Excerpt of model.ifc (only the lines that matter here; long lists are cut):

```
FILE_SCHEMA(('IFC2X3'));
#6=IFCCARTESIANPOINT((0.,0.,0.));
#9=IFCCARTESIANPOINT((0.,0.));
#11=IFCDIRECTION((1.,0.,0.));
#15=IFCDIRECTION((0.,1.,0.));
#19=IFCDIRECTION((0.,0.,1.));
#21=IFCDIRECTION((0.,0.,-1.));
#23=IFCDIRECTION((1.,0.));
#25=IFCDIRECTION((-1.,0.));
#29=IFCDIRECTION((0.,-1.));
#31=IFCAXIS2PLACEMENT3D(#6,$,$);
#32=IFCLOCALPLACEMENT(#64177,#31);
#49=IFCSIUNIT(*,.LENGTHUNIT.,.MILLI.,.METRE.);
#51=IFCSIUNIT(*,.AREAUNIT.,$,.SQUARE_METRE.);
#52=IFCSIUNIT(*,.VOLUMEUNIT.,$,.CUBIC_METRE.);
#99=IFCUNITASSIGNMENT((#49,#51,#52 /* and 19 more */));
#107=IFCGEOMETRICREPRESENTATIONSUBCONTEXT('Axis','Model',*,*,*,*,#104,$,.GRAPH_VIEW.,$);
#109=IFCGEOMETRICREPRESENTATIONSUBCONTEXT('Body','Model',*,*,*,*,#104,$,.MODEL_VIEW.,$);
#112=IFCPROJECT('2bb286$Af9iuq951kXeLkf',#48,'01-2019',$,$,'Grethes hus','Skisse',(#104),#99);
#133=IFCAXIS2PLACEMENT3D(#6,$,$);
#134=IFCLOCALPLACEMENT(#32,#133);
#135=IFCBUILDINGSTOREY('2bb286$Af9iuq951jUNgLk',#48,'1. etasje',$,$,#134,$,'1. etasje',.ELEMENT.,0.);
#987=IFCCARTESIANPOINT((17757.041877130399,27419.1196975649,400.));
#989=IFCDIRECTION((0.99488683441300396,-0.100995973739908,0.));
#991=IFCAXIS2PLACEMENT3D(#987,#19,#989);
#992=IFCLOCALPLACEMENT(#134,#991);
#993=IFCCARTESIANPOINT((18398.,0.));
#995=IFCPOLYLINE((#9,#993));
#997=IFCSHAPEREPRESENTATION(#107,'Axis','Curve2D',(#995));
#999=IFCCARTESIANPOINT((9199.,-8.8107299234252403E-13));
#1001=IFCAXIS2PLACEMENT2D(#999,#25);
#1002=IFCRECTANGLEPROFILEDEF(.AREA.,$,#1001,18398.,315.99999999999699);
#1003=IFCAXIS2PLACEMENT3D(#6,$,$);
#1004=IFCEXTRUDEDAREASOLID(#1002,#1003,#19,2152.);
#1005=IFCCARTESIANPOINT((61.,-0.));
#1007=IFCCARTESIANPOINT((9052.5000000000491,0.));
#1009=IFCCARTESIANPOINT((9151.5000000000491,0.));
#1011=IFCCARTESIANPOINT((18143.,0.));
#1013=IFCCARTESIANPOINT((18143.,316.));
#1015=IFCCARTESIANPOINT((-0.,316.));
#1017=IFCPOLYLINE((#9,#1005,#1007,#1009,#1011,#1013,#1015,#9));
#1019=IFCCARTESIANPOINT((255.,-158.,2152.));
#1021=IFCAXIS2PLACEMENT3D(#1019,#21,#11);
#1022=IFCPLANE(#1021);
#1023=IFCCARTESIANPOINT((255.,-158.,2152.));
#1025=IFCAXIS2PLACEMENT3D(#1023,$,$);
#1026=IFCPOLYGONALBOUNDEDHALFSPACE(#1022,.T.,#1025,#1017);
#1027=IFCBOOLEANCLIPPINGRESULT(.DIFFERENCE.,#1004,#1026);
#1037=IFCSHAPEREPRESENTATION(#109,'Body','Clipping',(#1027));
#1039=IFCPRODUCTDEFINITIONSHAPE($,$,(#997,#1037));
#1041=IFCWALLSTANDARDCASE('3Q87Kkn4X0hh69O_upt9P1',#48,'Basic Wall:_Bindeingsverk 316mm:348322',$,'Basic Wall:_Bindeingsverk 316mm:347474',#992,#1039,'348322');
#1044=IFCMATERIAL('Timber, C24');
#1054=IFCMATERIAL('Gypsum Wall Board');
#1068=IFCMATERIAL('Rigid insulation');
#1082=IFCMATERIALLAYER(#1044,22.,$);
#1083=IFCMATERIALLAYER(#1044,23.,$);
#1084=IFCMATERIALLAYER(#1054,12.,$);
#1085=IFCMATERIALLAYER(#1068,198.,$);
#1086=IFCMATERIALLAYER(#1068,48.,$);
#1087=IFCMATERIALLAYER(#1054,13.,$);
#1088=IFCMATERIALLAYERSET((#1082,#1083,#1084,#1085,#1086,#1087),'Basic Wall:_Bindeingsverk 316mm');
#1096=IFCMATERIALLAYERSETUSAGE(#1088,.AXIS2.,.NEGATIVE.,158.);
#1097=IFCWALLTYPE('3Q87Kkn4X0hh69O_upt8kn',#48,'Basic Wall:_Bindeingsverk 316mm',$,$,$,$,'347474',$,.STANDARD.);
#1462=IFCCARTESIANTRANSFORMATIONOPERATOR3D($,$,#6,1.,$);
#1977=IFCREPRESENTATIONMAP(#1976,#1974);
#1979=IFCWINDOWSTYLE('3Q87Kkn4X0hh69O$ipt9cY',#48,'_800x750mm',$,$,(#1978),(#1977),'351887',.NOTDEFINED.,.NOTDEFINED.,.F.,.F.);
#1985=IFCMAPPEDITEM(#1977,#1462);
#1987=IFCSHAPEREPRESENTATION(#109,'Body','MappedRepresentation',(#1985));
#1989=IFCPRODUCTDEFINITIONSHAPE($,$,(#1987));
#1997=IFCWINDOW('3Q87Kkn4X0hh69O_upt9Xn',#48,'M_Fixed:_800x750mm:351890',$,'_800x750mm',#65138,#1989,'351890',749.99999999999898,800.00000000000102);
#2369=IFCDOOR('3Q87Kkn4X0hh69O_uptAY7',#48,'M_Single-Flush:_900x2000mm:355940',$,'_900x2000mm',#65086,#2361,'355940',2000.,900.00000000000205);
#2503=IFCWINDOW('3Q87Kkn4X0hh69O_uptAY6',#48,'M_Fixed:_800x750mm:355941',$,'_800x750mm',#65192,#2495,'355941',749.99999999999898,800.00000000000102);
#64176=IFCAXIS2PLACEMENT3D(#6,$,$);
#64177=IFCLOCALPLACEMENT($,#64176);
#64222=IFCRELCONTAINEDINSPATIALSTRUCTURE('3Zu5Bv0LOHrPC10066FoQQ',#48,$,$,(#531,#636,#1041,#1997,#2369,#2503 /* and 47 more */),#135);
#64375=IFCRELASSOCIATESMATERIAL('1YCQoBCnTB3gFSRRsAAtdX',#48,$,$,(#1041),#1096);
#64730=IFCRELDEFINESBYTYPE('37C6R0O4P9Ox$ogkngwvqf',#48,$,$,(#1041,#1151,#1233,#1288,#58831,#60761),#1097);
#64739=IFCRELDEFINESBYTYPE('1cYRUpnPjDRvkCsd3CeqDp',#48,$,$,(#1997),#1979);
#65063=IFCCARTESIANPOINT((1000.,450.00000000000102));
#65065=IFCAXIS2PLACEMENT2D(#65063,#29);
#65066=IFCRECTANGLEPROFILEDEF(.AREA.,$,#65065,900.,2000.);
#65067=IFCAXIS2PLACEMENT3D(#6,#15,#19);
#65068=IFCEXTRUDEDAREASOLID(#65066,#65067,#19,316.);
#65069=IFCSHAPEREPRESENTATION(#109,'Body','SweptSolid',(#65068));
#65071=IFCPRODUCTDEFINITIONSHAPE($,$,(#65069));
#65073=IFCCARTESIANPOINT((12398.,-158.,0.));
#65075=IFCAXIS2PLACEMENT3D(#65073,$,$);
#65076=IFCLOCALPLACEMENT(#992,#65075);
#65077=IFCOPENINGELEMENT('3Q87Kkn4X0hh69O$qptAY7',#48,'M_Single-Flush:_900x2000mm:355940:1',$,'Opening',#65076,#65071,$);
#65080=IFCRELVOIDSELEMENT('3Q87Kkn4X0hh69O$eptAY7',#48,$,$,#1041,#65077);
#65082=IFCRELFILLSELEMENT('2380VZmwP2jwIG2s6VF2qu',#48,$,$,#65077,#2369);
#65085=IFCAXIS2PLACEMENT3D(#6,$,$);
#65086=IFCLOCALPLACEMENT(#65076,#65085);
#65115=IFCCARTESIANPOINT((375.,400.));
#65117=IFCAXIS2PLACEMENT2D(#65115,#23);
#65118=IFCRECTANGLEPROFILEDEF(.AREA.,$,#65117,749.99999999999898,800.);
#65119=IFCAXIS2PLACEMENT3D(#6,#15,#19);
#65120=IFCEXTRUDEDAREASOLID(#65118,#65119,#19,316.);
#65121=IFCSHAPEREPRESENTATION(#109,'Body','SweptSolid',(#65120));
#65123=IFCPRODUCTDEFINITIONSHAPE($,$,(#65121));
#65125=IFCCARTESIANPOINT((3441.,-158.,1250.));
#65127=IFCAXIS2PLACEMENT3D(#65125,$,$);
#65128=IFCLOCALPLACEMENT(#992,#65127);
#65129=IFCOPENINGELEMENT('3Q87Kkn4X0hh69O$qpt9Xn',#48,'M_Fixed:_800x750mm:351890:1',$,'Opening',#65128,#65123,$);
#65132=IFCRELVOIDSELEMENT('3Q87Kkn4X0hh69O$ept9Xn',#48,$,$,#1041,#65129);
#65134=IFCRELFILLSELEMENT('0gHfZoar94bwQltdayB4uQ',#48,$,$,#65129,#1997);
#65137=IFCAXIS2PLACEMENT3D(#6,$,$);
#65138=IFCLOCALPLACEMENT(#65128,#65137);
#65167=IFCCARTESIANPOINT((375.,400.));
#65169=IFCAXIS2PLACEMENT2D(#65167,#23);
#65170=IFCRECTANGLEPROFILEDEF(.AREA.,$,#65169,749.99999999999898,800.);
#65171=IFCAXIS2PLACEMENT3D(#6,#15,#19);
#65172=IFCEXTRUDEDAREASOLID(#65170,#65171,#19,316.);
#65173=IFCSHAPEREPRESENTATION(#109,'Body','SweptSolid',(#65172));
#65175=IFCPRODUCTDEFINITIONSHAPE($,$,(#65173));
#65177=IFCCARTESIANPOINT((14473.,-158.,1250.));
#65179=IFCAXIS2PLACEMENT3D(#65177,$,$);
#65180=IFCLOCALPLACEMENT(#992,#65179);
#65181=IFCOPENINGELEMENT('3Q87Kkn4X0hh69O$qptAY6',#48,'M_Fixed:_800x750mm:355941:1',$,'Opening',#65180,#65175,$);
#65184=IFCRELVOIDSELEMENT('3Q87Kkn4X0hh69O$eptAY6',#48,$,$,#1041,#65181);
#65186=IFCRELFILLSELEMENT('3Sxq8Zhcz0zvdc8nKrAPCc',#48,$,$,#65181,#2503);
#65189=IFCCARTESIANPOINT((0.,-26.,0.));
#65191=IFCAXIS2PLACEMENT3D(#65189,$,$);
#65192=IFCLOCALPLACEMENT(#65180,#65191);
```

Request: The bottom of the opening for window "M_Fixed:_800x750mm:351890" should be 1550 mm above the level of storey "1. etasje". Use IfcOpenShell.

```python
import numpy as np
import ifcopenshell
import ifcopenshell.api.geometry
import ifcopenshell.geom
import ifcopenshell.util.element
import ifcopenshell.util.placement
import ifcopenshell.util.shape
import ifcopenshell.util.unit

model = ifcopenshell.open("model.ifc")
unit_scale = ifcopenshell.util.unit.calculate_unit_scale(model)

window = model.by_guid("3Q87Kkn4X0hh69O_upt9Xn")
opening = window.FillsVoids[0].RelatingOpeningElement
storey = ifcopenshell.util.element.get_container(window, ifc_class="IfcBuildingStorey")
level = ifcopenshell.util.placement.get_local_placement(storey.ObjectPlacement)[2, 3]

# The opening's origin need not be at the sill, so measure its lowest point.
shape = ifcopenshell.geom.create_shape(ifcopenshell.geom.settings(), opening)
bottom = ifcopenshell.util.shape.get_shape_bottom_elevation(shape, shape.geometry) / unit_scale
dz = level + 1.55 / unit_scale - bottom

shift = np.array([0.0, 0.0, dz])
# The window is placed relative to its opening, so it follows when the opening moves.
matrix = ifcopenshell.util.placement.get_local_placement(opening.ObjectPlacement)
matrix[:3, 3] += shift
ifcopenshell.api.geometry.edit_object_placement(
    model, product=opening, matrix=matrix, is_si=False, should_transform_children=True
)

print(f"moved by {dz * unit_scale:+.3f} m")

model.write("model_v2.ifc")
```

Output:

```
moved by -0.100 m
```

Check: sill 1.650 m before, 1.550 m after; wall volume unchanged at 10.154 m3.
